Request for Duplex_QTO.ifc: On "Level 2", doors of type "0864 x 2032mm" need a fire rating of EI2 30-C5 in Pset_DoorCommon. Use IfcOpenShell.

First a look at what the model holds.

```python
import ifcopenshell
import ifcopenshell.util.element

model = ifcopenshell.open("Duplex_QTO.ifc")
print(model.schema)
storey = next(s for s in model.by_type("IfcBuildingStorey") if s.Name == "Level 2")
doors = [e for e in ifcopenshell.util.element.get_decomposition(storey) if e.is_a("IfcDoor")]
seen = {}
for e in doors:
    element_type = ifcopenshell.util.element.get_type(e)
    key = (element_type.Name if element_type != e and element_type else None, ifcopenshell.util.element.get_pset(e, "Pset_DoorCommon", "FireRating"))
    seen[key] = seen.get(key, 0) + 1
for (name, value), count in sorted(seen.items(), key=str):
    print(count, "x", name, "|", value)
```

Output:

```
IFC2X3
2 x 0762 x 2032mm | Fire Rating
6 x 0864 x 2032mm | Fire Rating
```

```python
import ifcopenshell
import ifcopenshell.api.pset
import ifcopenshell.util.element

model = ifcopenshell.open("Duplex_QTO.ifc")

storey = next(s for s in model.by_type("IfcBuildingStorey") if s.Name == "Level 2")
doors = [e for e in ifcopenshell.util.element.get_decomposition(storey) if e.is_a("IfcDoor")]

count = 0
for e in doors:
    element_type = ifcopenshell.util.element.get_type(e)
    if element_type in (None, e) or element_type.Name != "0864 x 2032mm":
        continue
    # add_pset returns the element's existing set when there is one.
    pset = ifcopenshell.api.pset.add_pset(model, product=e, name="Pset_DoorCommon")
    ifcopenshell.api.pset.edit_pset(model, pset=pset, properties={"FireRating": "EI2 30-C5"})
    count += 1

print(count, "doors updated")

model.write("Duplex_QTO_edited.ifc")
```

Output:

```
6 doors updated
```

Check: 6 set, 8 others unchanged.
